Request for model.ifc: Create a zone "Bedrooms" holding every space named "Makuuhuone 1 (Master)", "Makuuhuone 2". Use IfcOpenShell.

First a look at what the model holds.

```python
import ifcopenshell

model = ifcopenshell.open("model.ifc")
print(model.schema)
seen = {}
for space in model.by_type("IfcSpace"):
    seen[space.LongName] = seen.get(space.LongName, 0) + 1
for name, count in sorted(seen.items(), key=str):
    print(count, "x", name)
print("zones:", [z.Name for z in model.by_type("IfcZone")][:20])
```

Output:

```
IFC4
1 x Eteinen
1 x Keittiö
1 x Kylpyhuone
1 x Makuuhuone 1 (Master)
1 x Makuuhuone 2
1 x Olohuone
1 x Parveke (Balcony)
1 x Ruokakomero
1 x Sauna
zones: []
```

```python
import ifcopenshell
import ifcopenshell.api.group
import ifcopenshell.api.root

model = ifcopenshell.open("model.ifc")

names = {"Makuuhuone 1 (Master)", "Makuuhuone 2"}
spaces = [s for s in model.by_type("IfcSpace") if s.LongName in names]

zone = ifcopenshell.api.root.create_entity(model, ifc_class="IfcZone", name="Bedrooms")
ifcopenshell.api.group.assign_group(model, products=spaces, group=zone)
print(len(spaces), "spaces in", zone.Name)

model.write("model-out.ifc")
```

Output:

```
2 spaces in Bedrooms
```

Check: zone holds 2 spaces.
